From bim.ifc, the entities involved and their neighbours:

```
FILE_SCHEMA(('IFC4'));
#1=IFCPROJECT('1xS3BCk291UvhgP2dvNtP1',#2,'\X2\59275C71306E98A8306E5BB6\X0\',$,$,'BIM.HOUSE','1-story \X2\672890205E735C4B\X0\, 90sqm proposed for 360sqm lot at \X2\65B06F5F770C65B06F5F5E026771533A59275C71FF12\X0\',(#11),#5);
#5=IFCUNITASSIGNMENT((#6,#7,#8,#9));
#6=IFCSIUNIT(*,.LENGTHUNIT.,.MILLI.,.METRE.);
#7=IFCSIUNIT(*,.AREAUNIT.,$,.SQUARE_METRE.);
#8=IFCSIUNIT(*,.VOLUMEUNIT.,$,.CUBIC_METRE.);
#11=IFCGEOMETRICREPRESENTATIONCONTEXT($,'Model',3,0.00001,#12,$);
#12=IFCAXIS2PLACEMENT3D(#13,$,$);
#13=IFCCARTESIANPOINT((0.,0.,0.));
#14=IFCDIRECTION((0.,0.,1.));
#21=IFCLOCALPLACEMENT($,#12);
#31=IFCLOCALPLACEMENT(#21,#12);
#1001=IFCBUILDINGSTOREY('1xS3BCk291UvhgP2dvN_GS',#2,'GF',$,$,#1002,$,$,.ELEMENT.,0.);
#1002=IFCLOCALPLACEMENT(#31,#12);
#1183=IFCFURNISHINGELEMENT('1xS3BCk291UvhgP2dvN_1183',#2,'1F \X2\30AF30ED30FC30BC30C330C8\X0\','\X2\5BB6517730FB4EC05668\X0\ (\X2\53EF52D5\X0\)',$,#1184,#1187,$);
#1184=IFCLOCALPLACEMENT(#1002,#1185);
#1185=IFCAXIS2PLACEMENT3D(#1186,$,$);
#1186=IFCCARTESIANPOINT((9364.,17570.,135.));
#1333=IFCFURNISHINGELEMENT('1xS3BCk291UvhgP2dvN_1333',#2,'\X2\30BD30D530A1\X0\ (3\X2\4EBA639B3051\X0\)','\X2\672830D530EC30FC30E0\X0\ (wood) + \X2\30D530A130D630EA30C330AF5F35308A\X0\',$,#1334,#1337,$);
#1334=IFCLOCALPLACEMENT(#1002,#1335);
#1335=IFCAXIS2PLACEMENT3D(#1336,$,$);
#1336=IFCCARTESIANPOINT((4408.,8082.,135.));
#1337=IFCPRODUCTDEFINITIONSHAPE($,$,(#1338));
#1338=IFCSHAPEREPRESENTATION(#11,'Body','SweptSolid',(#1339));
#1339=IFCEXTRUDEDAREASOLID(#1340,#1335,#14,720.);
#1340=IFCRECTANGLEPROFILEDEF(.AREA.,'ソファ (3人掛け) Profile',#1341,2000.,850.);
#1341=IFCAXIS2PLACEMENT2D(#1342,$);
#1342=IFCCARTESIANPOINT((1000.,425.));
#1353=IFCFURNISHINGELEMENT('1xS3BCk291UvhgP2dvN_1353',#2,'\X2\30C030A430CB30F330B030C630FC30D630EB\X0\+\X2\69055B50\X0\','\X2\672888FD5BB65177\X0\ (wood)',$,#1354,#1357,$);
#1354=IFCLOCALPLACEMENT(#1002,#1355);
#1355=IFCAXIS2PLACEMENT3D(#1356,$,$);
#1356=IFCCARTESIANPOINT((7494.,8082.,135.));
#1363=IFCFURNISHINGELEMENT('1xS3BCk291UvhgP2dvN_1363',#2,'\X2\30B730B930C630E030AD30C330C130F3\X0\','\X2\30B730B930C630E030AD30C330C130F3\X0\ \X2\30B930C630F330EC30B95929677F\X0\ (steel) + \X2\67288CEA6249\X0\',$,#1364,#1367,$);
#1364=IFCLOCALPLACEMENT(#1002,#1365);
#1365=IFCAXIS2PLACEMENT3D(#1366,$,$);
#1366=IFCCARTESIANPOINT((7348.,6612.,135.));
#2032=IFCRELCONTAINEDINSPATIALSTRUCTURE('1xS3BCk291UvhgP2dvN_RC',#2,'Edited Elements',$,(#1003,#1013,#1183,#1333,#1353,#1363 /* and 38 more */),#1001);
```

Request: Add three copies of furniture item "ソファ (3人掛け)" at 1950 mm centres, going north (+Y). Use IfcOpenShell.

```python
import numpy as np
import ifcopenshell
import ifcopenshell.api.geometry
import ifcopenshell.api.root
import ifcopenshell.util.element
import ifcopenshell.util.placement

model = ifcopenshell.open("bim.ifc")


def reuse_history(source, copy):
    """copy_class also copies each property set's owner history, people and application; keep the originals."""
    for rel in copy.IsDefinedBy:
        if rel.is_a("IfcRelDefinesByProperties") and (history := rel.RelatingPropertyDefinition.OwnerHistory):
            rel.RelatingPropertyDefinition.OwnerHistory = source.OwnerHistory
            ifcopenshell.util.element.remove_deep2(model, history)


source = model.by_guid("1xS3BCk291UvhgP2dvN_1333")
base = ifcopenshell.util.placement.get_local_placement(source.ObjectPlacement)
step = np.array([0.0, 1.0, 0.0]) * 1950.0

for i in range(1, 4):
    copy = ifcopenshell.api.root.copy_class(model, product=source)
    copy.Representation = ifcopenshell.util.element.copy_deep(
        model, source.Representation, exclude=["IfcGeometricRepresentationContext", "IfcRepresentationMap"]
    )
    reuse_history(source, copy)
    matrix = base.copy()
    matrix[:3, 3] += i * step
    print("added at", matrix[:3, 3].round(3) + 0.0)
    ifcopenshell.api.geometry.edit_object_placement(model, product=copy, matrix=matrix, is_si=False)

model.write("bim_edited.ifc")
```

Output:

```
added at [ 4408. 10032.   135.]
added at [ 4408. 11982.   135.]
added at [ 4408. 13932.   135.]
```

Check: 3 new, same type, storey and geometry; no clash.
